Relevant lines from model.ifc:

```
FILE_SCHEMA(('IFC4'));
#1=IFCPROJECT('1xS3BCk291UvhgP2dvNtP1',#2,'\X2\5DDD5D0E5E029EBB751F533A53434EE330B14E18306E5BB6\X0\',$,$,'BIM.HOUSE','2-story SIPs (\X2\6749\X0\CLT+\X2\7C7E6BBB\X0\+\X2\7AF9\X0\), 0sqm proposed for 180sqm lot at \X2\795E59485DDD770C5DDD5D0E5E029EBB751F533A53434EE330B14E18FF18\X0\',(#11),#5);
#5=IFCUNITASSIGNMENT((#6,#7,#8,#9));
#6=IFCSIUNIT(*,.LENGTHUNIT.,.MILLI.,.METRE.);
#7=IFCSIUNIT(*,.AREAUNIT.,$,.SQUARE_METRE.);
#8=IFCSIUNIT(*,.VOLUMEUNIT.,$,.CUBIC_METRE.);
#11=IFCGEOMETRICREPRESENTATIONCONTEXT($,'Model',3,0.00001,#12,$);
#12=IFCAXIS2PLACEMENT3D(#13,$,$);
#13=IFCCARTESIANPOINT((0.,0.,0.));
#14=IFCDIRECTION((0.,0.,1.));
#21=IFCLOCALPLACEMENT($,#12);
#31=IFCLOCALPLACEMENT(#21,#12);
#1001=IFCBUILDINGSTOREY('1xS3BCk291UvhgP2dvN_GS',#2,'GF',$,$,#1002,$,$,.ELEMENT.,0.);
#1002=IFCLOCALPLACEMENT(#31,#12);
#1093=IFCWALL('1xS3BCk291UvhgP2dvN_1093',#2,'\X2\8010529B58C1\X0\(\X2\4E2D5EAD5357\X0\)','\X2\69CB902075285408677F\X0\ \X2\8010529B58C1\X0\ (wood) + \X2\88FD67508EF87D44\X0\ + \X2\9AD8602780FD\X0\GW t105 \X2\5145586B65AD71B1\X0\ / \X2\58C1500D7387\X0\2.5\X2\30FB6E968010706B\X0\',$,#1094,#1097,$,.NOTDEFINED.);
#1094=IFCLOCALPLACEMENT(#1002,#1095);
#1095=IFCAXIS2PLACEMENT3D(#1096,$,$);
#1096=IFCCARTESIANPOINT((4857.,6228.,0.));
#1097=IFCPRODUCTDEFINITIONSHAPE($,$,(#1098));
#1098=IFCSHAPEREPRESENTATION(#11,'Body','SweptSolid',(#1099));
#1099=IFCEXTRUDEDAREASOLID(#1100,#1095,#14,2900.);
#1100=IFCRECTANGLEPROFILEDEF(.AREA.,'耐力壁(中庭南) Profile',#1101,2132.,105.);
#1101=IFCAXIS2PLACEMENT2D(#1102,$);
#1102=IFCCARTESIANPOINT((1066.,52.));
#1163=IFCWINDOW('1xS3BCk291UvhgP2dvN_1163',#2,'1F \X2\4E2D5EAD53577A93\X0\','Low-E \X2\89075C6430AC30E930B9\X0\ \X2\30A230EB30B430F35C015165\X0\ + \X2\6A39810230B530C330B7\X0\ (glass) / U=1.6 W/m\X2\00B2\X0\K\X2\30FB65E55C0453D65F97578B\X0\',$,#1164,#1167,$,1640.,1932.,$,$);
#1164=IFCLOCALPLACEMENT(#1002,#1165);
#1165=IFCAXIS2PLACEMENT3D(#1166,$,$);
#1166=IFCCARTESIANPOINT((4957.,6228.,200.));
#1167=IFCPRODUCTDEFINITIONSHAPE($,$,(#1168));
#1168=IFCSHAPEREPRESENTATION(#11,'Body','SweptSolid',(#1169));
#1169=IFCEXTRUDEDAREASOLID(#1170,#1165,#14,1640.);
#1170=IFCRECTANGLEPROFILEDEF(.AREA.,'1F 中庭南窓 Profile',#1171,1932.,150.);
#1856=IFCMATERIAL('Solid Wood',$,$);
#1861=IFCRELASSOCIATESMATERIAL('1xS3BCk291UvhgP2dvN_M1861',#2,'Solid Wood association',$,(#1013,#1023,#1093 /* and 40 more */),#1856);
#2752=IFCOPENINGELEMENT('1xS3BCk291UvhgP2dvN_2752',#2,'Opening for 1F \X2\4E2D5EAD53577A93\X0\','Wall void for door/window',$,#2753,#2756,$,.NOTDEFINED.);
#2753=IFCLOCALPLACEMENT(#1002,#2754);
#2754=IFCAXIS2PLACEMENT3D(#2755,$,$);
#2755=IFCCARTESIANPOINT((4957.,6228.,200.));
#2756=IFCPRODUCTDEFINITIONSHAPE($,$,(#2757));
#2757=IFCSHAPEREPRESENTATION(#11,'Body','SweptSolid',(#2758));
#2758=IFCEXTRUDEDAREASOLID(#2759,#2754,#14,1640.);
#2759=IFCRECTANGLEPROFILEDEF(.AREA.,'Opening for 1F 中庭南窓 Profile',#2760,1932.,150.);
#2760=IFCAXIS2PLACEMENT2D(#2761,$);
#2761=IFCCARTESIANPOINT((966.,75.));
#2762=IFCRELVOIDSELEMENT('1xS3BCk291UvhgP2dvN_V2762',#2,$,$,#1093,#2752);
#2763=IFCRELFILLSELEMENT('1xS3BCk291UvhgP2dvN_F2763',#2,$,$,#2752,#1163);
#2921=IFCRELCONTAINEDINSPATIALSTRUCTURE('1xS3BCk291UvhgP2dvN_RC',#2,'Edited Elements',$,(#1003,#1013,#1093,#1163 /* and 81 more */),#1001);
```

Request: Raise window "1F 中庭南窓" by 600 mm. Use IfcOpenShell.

```python
import numpy as np
import ifcopenshell
import ifcopenshell.api.geometry
import ifcopenshell.util.placement
import ifcopenshell.util.unit

model = ifcopenshell.open("model.ifc")
unit_scale = ifcopenshell.util.unit.calculate_unit_scale(model)

window = model.by_guid("1xS3BCk291UvhgP2dvN_1163")
opening = window.FillsVoids[0].RelatingOpeningElement
dz = 600.0

shift = np.array([0.0, 0.0, dz])
# The window is not placed relative to its opening, so move both.
for product in (opening, window):
    matrix = ifcopenshell.util.placement.get_local_placement(product.ObjectPlacement)
    matrix[:3, 3] += shift
    ifcopenshell.api.geometry.edit_object_placement(model, product=product, matrix=matrix, is_si=False)

print(f"moved by {dz * unit_scale:+.3f} m")

model.write("model_edited.ifc")
```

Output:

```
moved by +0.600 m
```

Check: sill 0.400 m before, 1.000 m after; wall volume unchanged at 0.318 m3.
